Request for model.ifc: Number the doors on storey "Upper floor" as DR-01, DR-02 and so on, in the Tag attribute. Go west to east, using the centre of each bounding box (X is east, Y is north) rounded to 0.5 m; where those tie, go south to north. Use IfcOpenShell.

First a look at what the model holds.

```python
import ifcopenshell
import ifcopenshell.util.element
import ifcopenshell.util.placement

model = ifcopenshell.open("model.ifc")
print(model.schema)
storey = next(s for s in model.by_type("IfcBuildingStorey") if s.Name == "Upper floor")
doors = [e for e in ifcopenshell.util.element.get_decomposition(storey) if e.is_a("IfcDoor")]
for e in sorted(doors, key=lambda e: e.id()):
    origin = ifcopenshell.util.placement.get_local_placement(e.ObjectPlacement)[:3, 3]
    print(e.id(), e.Tag, e.Name, origin.round(2) + 0.0, sep=" | ")
```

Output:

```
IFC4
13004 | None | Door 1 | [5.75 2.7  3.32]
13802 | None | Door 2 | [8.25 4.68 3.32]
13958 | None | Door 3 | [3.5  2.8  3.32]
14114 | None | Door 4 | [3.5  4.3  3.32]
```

```python
import ifcopenshell
import ifcopenshell.geom
import ifcopenshell.util.element
import ifcopenshell.util.shape

model = ifcopenshell.open("model.ifc")
settings = ifcopenshell.geom.settings()
settings.set("use-world-coords", True)


def centre(element):
    shape = ifcopenshell.geom.create_shape(settings, element)
    return ifcopenshell.util.shape.get_bbox_centroid(shape.geometry)


storey = next(s for s in model.by_type("IfcBuildingStorey") if s.Name == "Upper floor")
doors = [e for e in ifcopenshell.util.element.get_decomposition(storey) if e.is_a("IfcDoor")]

# Insertion points can sit at a corner or the storey origin, so sort by the geometry (in metres).
centres = {e: centre(e) for e in doors}
doors.sort(key=lambda e: (round(centres[e][0] / 0.5), centres[e][1]))

for i, e in enumerate(doors, start=1):
    number = f"DR-{i:02d}"
    e.Tag = number
    print(e.id(), number)

model.write("model_updated.ifc")
```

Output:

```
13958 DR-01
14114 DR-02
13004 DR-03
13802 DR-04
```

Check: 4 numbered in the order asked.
